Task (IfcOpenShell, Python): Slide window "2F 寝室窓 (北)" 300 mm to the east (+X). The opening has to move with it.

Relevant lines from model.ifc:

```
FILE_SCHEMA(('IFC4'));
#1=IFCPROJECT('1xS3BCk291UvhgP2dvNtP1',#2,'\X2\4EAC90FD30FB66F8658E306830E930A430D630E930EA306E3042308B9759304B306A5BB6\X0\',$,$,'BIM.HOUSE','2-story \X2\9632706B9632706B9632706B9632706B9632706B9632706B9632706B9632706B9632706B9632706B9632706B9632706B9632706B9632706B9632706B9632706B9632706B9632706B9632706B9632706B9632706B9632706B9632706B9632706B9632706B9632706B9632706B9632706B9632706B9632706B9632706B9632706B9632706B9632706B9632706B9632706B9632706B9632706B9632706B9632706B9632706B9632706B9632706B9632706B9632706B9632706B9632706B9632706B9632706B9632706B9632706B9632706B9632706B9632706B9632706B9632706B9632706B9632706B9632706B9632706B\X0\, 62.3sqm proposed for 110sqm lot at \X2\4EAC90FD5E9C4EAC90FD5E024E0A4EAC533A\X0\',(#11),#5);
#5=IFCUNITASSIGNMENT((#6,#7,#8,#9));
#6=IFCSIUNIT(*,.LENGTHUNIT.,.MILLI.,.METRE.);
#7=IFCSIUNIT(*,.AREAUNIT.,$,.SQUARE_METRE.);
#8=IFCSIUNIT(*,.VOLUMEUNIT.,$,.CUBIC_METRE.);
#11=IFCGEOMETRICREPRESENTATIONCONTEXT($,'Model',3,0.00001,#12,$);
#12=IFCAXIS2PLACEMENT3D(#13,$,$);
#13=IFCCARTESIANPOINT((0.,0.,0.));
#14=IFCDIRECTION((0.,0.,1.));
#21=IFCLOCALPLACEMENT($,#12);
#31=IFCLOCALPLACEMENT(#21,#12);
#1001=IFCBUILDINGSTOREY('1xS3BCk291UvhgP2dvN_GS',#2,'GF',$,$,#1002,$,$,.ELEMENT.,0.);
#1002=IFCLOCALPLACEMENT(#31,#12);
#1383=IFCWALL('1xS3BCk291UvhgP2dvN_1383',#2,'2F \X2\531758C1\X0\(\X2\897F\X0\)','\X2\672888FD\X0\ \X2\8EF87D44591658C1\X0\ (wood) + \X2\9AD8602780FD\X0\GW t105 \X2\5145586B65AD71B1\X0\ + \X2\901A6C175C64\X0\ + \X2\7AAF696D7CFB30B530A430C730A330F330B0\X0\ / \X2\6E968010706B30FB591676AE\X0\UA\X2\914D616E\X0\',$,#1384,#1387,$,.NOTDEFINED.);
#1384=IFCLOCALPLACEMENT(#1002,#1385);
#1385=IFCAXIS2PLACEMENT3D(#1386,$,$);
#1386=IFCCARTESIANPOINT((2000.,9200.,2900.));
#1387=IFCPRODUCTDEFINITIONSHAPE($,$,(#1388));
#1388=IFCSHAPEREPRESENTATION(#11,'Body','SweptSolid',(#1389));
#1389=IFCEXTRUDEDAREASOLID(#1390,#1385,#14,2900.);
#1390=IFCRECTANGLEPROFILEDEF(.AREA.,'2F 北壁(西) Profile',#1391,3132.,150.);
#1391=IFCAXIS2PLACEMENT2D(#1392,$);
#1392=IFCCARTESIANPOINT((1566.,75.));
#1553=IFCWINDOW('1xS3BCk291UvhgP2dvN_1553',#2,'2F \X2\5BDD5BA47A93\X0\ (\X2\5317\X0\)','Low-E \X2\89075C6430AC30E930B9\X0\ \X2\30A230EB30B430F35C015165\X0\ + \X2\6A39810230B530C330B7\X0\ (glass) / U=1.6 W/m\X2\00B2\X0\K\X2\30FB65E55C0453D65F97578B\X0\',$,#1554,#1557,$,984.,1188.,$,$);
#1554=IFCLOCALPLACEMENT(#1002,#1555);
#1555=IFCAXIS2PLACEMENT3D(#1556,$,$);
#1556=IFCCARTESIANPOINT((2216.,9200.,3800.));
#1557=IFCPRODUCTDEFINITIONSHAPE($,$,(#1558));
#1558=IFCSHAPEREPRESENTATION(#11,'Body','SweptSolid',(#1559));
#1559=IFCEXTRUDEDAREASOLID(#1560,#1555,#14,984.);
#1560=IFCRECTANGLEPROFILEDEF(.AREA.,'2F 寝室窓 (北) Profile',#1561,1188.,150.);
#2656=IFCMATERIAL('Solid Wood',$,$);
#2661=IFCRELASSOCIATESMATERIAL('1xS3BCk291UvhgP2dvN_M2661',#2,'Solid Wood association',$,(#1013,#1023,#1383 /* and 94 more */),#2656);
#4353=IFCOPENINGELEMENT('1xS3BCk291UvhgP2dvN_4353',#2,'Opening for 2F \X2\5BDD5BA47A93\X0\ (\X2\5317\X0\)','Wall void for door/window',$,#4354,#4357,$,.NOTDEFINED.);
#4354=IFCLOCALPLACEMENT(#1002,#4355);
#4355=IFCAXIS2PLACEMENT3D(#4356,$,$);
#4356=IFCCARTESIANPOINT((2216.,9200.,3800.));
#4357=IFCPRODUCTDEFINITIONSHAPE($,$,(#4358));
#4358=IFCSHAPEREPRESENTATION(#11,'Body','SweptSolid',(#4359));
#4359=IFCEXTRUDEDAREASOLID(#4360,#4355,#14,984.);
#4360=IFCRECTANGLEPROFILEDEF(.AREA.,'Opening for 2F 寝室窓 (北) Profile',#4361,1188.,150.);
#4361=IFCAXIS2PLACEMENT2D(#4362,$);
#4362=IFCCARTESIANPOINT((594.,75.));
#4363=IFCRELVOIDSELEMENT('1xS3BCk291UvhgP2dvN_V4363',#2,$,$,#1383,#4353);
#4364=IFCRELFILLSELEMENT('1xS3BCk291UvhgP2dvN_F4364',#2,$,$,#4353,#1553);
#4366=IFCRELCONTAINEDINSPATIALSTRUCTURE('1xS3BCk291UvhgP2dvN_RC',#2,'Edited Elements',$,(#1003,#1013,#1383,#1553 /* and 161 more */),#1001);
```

```python
import ifcopenshell
import ifcopenshell.api.geometry
import ifcopenshell.util.placement

model = ifcopenshell.open("model.ifc")

window = model.by_id(1553)
opening = window.FillsVoids[0].RelatingOpeningElement
wall = opening.VoidsElements[0].RelatingBuildingElement

wall_matrix = ifcopenshell.util.placement.get_local_placement(wall.ObjectPlacement)
shift = wall_matrix[:3, 0] * 300.0
before = ifcopenshell.util.placement.get_local_placement(window.ObjectPlacement)[:3, 3].copy()

# The window is not placed relative to its opening, so move both.
for product in (opening, window):
    matrix = ifcopenshell.util.placement.get_local_placement(product.ObjectPlacement)
    matrix[:3, 3] += shift
    ifcopenshell.api.geometry.edit_object_placement(model, product=product, matrix=matrix, is_si=False)

after = ifcopenshell.util.placement.get_local_placement(window.ObjectPlacement)[:3, 3]
print("window moved by", (after - before).round(3) + 0.0)

model.write("model_v2.ifc")
```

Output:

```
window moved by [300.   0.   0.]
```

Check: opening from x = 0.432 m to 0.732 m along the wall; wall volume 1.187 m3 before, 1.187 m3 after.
